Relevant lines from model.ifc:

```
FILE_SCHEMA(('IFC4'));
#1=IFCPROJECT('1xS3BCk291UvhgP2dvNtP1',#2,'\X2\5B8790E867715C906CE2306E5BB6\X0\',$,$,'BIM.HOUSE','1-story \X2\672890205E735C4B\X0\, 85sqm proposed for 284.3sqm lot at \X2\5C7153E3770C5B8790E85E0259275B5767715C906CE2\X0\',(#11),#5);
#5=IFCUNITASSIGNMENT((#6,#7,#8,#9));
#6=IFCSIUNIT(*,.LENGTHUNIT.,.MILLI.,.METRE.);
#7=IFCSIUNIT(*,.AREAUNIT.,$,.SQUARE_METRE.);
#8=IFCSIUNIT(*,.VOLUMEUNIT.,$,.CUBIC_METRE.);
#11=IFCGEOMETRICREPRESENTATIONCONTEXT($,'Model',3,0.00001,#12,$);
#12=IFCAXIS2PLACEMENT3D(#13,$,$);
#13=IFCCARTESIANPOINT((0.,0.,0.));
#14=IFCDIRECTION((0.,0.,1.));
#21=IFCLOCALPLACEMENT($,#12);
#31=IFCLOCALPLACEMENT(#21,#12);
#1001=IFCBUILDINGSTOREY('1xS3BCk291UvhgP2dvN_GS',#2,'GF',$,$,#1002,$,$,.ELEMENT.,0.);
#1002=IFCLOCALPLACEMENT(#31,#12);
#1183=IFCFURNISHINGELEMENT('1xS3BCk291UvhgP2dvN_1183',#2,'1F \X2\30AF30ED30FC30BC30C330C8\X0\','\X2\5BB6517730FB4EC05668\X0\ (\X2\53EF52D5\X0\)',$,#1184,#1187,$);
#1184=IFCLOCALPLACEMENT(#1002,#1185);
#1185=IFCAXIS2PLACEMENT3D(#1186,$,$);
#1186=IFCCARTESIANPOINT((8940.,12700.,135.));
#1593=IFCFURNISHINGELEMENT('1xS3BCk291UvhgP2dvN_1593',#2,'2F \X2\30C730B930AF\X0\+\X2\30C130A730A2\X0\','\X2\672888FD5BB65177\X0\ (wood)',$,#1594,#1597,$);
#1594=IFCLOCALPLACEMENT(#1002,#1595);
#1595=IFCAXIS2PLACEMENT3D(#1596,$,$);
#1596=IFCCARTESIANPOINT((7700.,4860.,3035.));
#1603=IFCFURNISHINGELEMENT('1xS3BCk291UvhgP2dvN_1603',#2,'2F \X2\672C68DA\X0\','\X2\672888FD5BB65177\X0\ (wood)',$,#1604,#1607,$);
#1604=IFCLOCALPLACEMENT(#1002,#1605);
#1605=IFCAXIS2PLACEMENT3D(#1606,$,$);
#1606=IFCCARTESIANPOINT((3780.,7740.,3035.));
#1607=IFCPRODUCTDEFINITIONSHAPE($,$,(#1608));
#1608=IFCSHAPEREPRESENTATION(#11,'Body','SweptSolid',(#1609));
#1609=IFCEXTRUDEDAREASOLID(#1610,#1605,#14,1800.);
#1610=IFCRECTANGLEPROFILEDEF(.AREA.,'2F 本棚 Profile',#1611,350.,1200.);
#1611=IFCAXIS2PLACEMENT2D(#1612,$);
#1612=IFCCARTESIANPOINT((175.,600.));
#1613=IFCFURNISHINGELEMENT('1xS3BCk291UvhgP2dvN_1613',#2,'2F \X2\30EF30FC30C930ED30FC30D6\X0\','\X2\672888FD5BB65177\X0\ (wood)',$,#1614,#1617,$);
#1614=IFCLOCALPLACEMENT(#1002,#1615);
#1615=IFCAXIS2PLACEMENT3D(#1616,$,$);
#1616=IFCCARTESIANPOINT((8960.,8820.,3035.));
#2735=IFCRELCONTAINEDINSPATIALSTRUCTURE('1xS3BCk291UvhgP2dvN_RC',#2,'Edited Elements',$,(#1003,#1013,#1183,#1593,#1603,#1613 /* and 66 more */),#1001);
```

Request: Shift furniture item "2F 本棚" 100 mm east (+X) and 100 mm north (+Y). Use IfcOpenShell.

```python
import ifcopenshell
import ifcopenshell.api.geometry
import ifcopenshell.util.placement
import ifcopenshell.util.unit

model = ifcopenshell.open("model.ifc")
unit_scale = ifcopenshell.util.unit.calculate_unit_scale(model)

item = model.by_guid("1xS3BCk291UvhgP2dvN_1603")
matrix = ifcopenshell.util.placement.get_local_placement(item.ObjectPlacement)
matrix[0, 3] += 0.1 / unit_scale
matrix[1, 3] += 0.1 / unit_scale
ifcopenshell.api.geometry.edit_object_placement(model, product=item, matrix=matrix, is_si=False)

print(ifcopenshell.util.placement.get_local_placement(item.ObjectPlacement).round(3) + 0.0)

model.write("model_edited.ifc")
```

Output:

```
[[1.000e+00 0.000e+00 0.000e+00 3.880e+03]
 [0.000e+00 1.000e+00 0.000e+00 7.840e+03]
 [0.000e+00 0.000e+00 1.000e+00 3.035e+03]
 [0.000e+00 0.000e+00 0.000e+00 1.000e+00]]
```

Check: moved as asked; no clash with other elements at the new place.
